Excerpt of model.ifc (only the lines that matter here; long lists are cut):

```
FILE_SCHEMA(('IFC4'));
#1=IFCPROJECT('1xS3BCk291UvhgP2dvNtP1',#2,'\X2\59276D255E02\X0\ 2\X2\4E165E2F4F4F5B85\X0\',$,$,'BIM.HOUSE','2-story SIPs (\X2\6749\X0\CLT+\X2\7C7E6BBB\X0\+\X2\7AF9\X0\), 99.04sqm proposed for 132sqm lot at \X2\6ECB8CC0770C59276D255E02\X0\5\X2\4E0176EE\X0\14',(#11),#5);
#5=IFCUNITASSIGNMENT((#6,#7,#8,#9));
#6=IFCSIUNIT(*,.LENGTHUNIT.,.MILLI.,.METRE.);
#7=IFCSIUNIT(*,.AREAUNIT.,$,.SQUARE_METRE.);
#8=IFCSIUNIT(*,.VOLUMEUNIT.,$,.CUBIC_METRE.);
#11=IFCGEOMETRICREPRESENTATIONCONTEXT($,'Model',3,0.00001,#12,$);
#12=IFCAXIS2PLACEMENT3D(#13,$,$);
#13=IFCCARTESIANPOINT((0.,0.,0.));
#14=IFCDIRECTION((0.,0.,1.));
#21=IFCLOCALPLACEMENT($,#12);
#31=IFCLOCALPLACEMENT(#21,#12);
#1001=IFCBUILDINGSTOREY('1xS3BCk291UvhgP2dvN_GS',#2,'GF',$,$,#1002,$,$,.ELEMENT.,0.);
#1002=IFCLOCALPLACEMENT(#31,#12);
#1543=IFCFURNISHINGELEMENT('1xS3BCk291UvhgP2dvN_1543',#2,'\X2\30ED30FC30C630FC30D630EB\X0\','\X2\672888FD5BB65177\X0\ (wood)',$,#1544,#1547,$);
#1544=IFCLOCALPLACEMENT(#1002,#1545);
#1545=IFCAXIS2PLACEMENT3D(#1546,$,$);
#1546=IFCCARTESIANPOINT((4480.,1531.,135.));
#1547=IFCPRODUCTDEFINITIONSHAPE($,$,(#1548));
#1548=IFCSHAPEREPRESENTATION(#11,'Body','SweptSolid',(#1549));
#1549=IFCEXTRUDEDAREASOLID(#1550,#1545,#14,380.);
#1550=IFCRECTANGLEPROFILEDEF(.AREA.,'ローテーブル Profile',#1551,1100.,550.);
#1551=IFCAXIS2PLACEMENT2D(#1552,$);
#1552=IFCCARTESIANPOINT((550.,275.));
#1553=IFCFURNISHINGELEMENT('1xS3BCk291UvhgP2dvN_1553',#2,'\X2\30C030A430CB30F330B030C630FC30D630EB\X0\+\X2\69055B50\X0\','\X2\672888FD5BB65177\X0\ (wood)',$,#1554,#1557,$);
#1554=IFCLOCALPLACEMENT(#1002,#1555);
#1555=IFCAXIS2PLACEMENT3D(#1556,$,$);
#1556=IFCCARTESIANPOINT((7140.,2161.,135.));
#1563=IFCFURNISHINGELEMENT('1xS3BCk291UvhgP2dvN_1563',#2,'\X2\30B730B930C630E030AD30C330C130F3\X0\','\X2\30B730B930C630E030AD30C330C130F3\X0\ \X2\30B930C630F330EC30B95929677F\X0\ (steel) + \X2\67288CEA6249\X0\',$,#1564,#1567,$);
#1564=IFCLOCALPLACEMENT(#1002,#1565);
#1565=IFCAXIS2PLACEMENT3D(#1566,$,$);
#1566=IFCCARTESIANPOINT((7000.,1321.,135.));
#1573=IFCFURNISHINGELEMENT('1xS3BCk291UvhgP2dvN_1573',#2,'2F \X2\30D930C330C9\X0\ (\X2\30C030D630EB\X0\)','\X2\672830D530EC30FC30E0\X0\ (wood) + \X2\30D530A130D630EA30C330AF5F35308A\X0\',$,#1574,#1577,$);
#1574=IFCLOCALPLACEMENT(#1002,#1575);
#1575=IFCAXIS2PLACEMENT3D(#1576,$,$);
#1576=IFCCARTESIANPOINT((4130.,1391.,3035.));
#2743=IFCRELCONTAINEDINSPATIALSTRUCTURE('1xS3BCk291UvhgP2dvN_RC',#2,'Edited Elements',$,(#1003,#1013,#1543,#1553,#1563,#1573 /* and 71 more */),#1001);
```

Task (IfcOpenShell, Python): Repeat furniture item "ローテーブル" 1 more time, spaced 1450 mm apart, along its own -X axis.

```python
import ifcopenshell
import ifcopenshell.api.geometry
import ifcopenshell.api.root
import ifcopenshell.util.element
import ifcopenshell.util.placement

model = ifcopenshell.open("model.ifc")


def reuse_history(source, copy):
    """copy_class also copies each property set's owner history, people and application; keep the originals."""
    for rel in copy.IsDefinedBy:
        if rel.is_a("IfcRelDefinesByProperties") and (history := rel.RelatingPropertyDefinition.OwnerHistory):
            rel.RelatingPropertyDefinition.OwnerHistory = source.OwnerHistory
            ifcopenshell.util.element.remove_deep2(model, history)


source = model.by_guid("1xS3BCk291UvhgP2dvN_1543")
base = ifcopenshell.util.placement.get_local_placement(source.ObjectPlacement)
step = -base[:3, 0] * 1450.0

for i in range(1, 2):
    copy = ifcopenshell.api.root.copy_class(model, product=source)
    copy.Representation = ifcopenshell.util.element.copy_deep(
        model, source.Representation, exclude=["IfcGeometricRepresentationContext", "IfcRepresentationMap"]
    )
    reuse_history(source, copy)
    matrix = base.copy()
    matrix[:3, 3] += i * step
    print("added at", matrix[:3, 3].round(3) + 0.0)
    ifcopenshell.api.geometry.edit_object_placement(model, product=copy, matrix=matrix, is_si=False)

model.write("model-out.ifc")
```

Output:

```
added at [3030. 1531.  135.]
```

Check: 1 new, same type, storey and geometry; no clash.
